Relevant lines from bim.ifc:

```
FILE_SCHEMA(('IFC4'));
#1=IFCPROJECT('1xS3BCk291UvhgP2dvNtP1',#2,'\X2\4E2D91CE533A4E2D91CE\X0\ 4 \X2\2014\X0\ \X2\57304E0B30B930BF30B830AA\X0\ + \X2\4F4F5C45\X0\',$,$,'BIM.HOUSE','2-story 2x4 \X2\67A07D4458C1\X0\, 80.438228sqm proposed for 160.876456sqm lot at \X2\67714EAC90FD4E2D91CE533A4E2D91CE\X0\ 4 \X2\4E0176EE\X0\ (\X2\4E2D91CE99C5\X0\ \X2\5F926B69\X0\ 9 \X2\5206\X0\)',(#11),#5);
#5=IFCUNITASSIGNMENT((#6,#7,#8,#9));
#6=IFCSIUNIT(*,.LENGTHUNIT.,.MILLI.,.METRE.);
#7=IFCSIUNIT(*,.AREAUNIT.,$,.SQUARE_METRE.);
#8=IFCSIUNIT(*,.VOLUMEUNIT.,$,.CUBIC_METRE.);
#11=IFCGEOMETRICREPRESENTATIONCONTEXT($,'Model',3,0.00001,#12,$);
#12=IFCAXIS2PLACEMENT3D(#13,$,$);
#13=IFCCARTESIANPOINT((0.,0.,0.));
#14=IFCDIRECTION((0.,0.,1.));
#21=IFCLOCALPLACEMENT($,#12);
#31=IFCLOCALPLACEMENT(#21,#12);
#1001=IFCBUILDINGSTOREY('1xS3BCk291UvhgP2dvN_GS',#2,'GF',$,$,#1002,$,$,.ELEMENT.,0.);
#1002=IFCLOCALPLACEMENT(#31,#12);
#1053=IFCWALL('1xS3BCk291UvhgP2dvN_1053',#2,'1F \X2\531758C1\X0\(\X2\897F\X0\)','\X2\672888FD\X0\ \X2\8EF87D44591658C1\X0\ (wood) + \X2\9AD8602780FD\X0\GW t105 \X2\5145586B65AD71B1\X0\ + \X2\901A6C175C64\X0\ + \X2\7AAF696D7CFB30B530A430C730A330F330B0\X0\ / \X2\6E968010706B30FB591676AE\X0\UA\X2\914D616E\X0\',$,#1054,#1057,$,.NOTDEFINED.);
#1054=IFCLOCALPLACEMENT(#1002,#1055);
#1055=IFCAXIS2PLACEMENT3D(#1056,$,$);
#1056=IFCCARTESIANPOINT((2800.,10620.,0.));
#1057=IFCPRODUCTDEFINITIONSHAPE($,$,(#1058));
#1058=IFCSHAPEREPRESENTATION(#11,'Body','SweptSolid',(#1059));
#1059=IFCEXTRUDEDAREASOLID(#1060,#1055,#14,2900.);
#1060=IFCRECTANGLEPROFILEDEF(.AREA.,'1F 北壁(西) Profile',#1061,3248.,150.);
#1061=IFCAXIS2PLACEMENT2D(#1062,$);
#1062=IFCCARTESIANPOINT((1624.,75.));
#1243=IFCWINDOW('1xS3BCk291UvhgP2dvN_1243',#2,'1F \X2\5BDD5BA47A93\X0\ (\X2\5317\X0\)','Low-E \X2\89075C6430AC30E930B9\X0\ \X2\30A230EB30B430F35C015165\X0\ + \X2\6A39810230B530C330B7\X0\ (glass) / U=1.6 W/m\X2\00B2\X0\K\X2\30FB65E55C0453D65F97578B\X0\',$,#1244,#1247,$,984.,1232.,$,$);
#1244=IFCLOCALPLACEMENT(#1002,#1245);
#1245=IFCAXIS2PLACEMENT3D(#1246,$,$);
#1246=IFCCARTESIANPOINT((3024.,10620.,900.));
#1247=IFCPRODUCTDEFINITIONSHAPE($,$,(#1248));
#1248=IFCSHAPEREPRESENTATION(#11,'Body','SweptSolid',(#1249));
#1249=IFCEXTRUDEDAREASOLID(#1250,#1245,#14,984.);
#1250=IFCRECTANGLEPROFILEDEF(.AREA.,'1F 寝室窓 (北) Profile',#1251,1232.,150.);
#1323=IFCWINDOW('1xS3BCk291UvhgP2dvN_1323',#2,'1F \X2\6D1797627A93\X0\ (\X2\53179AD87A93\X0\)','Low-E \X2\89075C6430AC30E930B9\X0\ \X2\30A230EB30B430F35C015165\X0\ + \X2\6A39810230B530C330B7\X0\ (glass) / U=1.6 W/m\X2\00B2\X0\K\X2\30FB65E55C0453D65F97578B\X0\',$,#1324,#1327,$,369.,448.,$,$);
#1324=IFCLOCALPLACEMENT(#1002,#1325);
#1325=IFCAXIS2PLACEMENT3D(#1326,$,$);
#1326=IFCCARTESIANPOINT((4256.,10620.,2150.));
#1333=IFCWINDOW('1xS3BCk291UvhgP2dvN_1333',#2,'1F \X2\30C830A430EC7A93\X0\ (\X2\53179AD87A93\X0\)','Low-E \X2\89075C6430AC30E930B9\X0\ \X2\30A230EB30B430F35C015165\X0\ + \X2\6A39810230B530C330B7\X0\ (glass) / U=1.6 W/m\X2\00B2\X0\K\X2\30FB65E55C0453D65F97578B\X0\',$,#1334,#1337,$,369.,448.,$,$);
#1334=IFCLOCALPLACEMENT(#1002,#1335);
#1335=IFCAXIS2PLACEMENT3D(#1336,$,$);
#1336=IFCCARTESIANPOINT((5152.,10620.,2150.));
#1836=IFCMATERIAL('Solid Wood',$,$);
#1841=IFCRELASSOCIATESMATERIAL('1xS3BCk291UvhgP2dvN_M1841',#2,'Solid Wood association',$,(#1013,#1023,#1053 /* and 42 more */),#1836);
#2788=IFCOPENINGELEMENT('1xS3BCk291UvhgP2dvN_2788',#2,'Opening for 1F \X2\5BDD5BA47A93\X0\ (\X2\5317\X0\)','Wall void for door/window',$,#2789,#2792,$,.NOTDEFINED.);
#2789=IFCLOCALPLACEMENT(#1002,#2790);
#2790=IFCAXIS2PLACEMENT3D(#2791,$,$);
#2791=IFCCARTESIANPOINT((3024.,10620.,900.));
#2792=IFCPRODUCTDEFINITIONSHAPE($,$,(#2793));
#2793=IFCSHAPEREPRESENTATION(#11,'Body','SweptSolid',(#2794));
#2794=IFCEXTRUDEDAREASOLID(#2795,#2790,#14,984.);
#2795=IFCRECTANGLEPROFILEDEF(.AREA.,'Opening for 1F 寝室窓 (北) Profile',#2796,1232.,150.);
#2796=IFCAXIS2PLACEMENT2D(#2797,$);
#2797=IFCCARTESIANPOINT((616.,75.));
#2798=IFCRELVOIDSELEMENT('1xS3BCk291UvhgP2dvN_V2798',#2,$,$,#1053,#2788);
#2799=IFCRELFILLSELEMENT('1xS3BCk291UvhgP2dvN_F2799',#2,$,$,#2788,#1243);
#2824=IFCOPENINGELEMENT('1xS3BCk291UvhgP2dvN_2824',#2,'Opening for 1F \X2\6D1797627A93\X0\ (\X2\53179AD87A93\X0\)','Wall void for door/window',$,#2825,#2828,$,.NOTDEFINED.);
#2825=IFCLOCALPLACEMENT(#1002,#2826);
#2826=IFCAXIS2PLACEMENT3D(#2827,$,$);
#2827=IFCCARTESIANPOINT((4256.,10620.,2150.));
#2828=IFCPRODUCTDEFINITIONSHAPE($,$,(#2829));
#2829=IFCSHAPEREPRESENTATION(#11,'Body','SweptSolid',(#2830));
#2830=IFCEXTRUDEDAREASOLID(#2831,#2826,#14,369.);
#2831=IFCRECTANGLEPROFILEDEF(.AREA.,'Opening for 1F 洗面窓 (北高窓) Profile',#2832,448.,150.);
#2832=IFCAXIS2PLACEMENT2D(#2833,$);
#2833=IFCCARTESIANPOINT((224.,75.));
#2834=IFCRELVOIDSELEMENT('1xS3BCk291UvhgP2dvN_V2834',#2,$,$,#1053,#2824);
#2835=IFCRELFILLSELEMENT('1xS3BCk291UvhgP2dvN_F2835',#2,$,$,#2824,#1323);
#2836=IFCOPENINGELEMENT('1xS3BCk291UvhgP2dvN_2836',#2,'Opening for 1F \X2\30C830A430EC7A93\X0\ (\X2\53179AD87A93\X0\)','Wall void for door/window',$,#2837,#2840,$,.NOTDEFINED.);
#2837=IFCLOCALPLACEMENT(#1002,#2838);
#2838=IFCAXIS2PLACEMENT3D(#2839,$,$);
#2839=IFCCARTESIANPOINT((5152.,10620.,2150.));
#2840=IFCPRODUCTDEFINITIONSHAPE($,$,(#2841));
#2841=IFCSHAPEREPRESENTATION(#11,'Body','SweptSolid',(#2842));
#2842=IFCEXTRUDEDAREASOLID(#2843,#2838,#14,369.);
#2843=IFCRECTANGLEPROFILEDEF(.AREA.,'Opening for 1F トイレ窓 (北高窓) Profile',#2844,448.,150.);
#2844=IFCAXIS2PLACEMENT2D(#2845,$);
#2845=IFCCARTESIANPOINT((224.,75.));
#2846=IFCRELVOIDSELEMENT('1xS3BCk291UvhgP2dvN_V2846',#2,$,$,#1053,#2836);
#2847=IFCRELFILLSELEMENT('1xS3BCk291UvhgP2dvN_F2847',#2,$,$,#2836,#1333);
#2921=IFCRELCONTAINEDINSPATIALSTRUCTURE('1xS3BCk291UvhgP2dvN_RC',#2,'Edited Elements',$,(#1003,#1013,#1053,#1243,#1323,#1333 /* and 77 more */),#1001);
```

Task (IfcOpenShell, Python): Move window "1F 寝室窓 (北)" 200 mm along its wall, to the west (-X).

```python
import ifcopenshell
import ifcopenshell.api.geometry
import ifcopenshell.util.placement
import ifcopenshell.util.unit

model = ifcopenshell.open("bim.ifc")
unit_scale = ifcopenshell.util.unit.calculate_unit_scale(model)

window = model.by_guid("1xS3BCk291UvhgP2dvN_1243")
opening = window.FillsVoids[0].RelatingOpeningElement
wall = opening.VoidsElements[0].RelatingBuildingElement

wall_matrix = ifcopenshell.util.placement.get_local_placement(wall.ObjectPlacement)
shift = wall_matrix[:3, 0] * -0.2 / unit_scale
before = ifcopenshell.util.placement.get_local_placement(window.ObjectPlacement)[:3, 3].copy()

# The window is not placed relative to its opening, so move both.
for product in (opening, window):
    matrix = ifcopenshell.util.placement.get_local_placement(product.ObjectPlacement)
    matrix[:3, 3] += shift
    ifcopenshell.api.geometry.edit_object_placement(model, product=product, matrix=matrix, is_si=False)

after = ifcopenshell.util.placement.get_local_placement(window.ObjectPlacement)[:3, 3]
print("window moved by", (after - before).round(3) + 0.0)

model.write("bim_v2.ifc")
```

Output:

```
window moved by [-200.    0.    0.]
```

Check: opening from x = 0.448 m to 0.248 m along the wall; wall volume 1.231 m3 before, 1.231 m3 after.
